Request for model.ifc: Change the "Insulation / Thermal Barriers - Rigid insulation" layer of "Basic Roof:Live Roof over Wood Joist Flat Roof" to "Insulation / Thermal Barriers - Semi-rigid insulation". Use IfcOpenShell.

First a look at what the model holds.

```python
import ifcopenshell
import ifcopenshell.util.element

model = ifcopenshell.open("model.ifc")
print(model.schema)
for layer_set in model.by_type("IfcMaterialLayerSet"):
    if layer_set.LayerSetName == "Basic Roof:Live Roof over Wood Joist Flat Roof":
        for layer in layer_set.MaterialLayers:
            print(layer.id(), layer.Material and layer.Material.Name, layer.LayerThickness, sep=" | ")
        print(len(ifcopenshell.util.element.get_elements_by_material(model, layer_set)), "elements and types use it")
print(sorted(m.Name for m in model.by_type("IfcMaterial") if m.Name)[:60])
```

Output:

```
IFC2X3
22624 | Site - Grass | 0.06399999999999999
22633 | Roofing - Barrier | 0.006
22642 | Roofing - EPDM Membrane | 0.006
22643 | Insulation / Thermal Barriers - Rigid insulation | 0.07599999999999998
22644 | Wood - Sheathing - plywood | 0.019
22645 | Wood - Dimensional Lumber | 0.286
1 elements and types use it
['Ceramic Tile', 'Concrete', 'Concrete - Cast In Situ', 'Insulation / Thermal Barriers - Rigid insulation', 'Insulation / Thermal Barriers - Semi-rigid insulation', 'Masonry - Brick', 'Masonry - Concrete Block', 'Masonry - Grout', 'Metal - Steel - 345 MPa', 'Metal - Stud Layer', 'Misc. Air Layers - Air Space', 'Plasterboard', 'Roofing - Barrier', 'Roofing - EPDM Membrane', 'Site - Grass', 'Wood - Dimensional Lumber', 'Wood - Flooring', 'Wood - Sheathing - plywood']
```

```python
import ifcopenshell
import ifcopenshell.api.material

model = ifcopenshell.open("model.ifc")

layer_set = next(s for s in model.by_type("IfcMaterialLayerSet") if s.LayerSetName == "Basic Roof:Live Roof over Wood Joist Flat Roof")
layer = next(l for l in layer_set.MaterialLayers if l.Material and l.Material.Name == "Insulation / Thermal Barriers - Rigid insulation")
material = next(m for m in model.by_type("IfcMaterial") if m.Name == "Insulation / Thermal Barriers - Semi-rigid insulation")

# Point this one layer at the other material; renaming the old one would change it everywhere.
ifcopenshell.api.material.edit_layer(model, layer=layer, attributes={}, material=material)

print([l.Material.Name if l.Material else None for l in layer_set.MaterialLayers])

model.write("model-out.ifc")
```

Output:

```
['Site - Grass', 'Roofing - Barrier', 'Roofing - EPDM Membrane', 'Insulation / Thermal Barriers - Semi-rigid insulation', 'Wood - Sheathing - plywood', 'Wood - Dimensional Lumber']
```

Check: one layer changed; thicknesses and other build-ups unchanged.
